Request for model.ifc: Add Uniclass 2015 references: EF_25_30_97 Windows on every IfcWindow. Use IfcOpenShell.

First a look at what the model holds.

```python
import ifcopenshell

model = ifcopenshell.open("model.ifc")
print(model.schema)
print("classifications:", [c.Name for c in model.by_type("IfcClassification")])
for ifc_class in ("IfcDoor", "IfcRoof", "IfcStair", "IfcWall", "IfcWindow"):
    print(ifc_class, len(model.by_type(ifc_class)))
```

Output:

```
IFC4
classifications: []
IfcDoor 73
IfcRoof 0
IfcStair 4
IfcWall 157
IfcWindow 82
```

```python
import ifcopenshell
import ifcopenshell.api.classification

model = ifcopenshell.open("model.ifc")

system = ifcopenshell.api.classification.add_classification(model, classification="Uniclass 2015")

codes = {
    "IfcWindow": ("EF_25_30_97", "Windows"),
}
for ifc_class, (code, name) in codes.items():
    products = model.by_type(ifc_class)
    ifcopenshell.api.classification.add_reference(
        model, products=products, classification=system, identification=code, name=name
    )
    print(code, len(products))

model.write("model_v2.ifc")
```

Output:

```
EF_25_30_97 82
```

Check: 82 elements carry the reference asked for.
